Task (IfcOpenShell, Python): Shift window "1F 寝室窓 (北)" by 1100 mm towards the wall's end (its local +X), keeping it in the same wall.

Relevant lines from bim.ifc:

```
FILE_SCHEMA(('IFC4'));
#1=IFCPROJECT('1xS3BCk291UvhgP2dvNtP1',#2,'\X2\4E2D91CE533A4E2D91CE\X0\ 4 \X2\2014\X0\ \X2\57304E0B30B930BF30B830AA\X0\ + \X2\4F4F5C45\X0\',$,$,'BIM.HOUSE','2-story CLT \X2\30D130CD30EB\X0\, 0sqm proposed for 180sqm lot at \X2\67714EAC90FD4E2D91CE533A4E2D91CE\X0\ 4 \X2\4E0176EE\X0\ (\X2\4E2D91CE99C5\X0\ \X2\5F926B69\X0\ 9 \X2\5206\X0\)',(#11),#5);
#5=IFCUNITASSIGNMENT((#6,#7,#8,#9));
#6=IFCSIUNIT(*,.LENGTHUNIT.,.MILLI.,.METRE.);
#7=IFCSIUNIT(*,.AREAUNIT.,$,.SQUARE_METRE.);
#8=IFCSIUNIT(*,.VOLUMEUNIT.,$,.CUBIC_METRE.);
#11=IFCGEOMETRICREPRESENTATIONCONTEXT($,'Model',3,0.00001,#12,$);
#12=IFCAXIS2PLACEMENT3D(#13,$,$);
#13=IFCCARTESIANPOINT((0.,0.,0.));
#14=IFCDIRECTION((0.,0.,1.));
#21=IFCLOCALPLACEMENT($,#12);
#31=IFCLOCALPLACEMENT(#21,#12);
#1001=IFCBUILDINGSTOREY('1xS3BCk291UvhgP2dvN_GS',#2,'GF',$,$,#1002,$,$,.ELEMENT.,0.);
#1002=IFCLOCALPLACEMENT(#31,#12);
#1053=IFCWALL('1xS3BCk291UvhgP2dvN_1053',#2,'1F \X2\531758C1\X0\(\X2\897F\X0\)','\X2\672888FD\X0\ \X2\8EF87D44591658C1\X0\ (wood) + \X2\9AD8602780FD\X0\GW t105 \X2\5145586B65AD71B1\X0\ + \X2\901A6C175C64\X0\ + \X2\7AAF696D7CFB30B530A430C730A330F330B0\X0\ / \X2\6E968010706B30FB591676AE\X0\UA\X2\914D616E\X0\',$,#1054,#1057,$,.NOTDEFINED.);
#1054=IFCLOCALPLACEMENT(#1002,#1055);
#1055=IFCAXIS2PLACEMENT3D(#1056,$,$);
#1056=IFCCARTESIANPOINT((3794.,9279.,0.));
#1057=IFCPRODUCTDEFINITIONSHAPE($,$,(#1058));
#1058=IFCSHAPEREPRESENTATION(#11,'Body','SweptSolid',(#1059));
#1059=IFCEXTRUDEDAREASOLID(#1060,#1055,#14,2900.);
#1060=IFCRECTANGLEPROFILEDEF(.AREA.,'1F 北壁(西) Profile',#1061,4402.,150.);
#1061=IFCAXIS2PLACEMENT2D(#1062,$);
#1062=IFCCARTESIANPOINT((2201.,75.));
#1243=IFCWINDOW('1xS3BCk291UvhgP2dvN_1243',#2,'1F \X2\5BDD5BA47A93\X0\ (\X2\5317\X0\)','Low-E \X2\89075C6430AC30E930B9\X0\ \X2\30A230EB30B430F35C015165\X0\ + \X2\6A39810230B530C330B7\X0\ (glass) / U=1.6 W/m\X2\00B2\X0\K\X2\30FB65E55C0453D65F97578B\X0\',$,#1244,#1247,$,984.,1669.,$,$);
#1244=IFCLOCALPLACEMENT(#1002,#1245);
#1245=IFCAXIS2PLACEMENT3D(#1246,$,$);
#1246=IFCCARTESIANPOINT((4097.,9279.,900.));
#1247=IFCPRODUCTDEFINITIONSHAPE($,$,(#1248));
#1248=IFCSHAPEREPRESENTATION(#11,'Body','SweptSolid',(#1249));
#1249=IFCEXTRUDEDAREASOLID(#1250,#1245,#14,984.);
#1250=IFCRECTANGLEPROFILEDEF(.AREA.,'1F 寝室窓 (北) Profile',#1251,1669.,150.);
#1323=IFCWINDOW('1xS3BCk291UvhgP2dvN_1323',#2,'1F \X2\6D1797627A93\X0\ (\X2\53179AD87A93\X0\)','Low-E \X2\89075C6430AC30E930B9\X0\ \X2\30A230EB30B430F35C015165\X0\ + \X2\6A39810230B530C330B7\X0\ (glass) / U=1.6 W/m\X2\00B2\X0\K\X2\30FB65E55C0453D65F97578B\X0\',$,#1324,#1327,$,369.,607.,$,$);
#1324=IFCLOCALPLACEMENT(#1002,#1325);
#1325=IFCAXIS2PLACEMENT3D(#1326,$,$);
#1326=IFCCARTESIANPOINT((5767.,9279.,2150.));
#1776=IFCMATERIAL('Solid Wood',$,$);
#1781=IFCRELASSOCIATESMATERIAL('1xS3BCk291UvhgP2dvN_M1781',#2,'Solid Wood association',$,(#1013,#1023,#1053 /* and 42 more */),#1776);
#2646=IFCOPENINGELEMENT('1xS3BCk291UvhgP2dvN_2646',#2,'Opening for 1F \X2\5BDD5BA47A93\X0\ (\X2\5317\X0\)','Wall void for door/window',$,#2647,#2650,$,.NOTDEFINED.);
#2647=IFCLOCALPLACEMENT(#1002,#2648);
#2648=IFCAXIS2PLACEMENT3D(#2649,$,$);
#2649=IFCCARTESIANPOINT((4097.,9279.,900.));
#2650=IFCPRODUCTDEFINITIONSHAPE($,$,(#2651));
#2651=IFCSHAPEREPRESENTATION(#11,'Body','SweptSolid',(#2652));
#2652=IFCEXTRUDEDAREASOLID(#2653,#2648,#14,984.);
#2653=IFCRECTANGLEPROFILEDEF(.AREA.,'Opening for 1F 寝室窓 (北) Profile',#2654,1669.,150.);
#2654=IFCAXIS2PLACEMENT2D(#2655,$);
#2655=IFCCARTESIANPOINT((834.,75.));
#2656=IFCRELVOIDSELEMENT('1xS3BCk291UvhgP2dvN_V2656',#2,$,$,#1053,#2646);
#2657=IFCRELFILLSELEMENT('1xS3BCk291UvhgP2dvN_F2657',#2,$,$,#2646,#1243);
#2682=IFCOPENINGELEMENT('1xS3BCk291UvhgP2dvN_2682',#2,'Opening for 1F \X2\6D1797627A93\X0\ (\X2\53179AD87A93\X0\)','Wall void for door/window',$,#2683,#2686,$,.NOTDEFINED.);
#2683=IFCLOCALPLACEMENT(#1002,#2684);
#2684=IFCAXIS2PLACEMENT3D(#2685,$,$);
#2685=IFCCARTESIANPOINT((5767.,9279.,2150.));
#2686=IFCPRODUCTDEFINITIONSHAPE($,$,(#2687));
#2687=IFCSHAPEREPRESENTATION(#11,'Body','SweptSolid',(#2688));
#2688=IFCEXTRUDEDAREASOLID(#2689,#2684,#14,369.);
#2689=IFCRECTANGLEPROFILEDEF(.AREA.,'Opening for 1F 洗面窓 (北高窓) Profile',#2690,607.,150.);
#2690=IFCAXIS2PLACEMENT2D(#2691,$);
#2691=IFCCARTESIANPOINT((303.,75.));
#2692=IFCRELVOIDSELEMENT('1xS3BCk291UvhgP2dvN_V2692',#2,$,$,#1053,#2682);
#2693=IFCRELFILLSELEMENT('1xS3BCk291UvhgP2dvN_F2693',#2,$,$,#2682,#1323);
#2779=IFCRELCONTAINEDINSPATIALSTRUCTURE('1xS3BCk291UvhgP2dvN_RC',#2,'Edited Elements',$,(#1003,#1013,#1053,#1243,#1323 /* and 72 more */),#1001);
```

```python
import ifcopenshell
import ifcopenshell.api.geometry
import ifcopenshell.util.placement
import ifcopenshell.util.unit

model = ifcopenshell.open("bim.ifc")
unit_scale = ifcopenshell.util.unit.calculate_unit_scale(model)

window = model.by_guid("1xS3BCk291UvhgP2dvN_1243")
opening = window.FillsVoids[0].RelatingOpeningElement
wall = opening.VoidsElements[0].RelatingBuildingElement

wall_matrix = ifcopenshell.util.placement.get_local_placement(wall.ObjectPlacement)
shift = wall_matrix[:3, 0] * 1.1 / unit_scale
before = ifcopenshell.util.placement.get_local_placement(window.ObjectPlacement)[:3, 3].copy()

# The window is not placed relative to its opening, so move both.
for product in (opening, window):
    matrix = ifcopenshell.util.placement.get_local_placement(product.ObjectPlacement)
    matrix[:3, 3] += shift
    ifcopenshell.api.geometry.edit_object_placement(model, product=product, matrix=matrix, is_si=False)

after = ifcopenshell.util.placement.get_local_placement(window.ObjectPlacement)[:3, 3]
print("window moved by", (after - before).round(3) + 0.0)

model.write("bim-out.ifc")
```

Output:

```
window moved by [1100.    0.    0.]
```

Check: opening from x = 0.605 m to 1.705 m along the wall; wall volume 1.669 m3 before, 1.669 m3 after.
